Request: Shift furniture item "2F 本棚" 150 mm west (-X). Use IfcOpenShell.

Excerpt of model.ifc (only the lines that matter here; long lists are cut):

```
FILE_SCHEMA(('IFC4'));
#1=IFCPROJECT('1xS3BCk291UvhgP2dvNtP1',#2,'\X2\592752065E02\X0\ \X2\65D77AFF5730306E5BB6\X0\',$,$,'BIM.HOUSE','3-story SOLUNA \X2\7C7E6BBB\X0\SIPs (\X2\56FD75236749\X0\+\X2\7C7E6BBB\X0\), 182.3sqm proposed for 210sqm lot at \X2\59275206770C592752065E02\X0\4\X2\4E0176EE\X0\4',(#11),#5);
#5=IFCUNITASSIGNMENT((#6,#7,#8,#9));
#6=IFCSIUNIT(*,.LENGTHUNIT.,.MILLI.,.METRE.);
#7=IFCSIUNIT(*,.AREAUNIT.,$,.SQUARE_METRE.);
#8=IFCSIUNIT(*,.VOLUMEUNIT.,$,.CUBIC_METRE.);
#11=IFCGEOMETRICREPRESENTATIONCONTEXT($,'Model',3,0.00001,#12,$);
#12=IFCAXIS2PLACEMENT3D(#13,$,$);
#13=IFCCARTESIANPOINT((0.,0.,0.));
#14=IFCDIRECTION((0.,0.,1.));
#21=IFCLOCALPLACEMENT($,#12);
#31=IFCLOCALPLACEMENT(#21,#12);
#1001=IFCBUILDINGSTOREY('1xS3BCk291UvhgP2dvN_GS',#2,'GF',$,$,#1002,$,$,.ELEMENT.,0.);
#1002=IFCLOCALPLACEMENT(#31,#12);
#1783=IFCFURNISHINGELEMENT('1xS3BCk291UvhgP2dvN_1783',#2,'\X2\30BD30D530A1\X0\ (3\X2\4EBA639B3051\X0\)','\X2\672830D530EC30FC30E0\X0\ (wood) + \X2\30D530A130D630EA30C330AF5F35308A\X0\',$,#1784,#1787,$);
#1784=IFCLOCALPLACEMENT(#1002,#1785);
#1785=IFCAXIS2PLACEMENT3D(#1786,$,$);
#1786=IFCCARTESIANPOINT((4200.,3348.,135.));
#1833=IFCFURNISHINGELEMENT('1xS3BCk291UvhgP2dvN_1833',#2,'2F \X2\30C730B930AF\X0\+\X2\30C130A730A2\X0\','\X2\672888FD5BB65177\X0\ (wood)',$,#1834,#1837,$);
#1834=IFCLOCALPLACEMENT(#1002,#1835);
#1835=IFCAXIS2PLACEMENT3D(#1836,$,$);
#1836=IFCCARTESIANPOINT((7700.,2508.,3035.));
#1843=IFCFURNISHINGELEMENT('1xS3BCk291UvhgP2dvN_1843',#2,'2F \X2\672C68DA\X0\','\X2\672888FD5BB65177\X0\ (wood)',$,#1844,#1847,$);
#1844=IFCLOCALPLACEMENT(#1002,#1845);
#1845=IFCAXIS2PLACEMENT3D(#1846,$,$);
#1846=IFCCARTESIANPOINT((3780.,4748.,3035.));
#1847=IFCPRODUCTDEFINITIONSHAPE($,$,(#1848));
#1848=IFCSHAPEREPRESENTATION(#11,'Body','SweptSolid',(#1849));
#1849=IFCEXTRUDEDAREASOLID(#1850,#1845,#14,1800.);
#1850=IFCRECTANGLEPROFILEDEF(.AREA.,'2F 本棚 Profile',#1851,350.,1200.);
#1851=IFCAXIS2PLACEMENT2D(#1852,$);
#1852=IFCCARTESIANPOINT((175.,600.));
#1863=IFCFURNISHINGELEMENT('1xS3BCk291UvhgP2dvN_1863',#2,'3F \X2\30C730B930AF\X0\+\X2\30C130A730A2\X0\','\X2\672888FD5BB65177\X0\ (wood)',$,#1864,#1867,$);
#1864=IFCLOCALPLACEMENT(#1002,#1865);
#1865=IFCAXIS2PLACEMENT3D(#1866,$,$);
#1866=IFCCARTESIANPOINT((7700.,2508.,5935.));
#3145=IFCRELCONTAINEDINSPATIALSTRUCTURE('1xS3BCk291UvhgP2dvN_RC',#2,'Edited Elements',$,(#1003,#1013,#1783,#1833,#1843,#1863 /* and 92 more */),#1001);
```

```python
import ifcopenshell
import ifcopenshell.api.geometry
import ifcopenshell.util.placement
import ifcopenshell.util.unit

model = ifcopenshell.open("model.ifc")
unit_scale = ifcopenshell.util.unit.calculate_unit_scale(model)

item = model.by_guid("1xS3BCk291UvhgP2dvN_1843")
matrix = ifcopenshell.util.placement.get_local_placement(item.ObjectPlacement)
matrix[0, 3] -= 0.15 / unit_scale
ifcopenshell.api.geometry.edit_object_placement(model, product=item, matrix=matrix, is_si=False)

print(ifcopenshell.util.placement.get_local_placement(item.ObjectPlacement).round(3) + 0.0)

model.write("model_edited.ifc")
```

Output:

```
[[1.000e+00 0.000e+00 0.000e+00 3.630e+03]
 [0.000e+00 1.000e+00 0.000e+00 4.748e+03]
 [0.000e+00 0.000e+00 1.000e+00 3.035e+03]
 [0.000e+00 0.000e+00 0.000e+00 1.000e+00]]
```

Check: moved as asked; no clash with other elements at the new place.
